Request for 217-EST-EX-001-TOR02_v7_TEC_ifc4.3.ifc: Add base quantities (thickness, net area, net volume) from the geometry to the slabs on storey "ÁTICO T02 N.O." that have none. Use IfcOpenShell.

First a look at what the model holds.

```python
import ifcopenshell
import ifcopenshell.util.element
import ifcopenshell.util.unit

model = ifcopenshell.open("217-EST-EX-001-TOR02_v7_TEC_ifc4.3.ifc")
print(model.schema)
for unit_type in ("LENGTHUNIT", "AREAUNIT", "VOLUMEUNIT"):
    print(unit_type, ifcopenshell.util.unit.calculate_unit_scale(model, unit_type))
storey = next(s for s in model.by_type("IfcBuildingStorey") if s.Name == "ÁTICO T02 N.O.")
slabs = [e for e in ifcopenshell.util.element.get_decomposition(storey) if e.is_a("IfcSlab")]
for e in sorted(slabs, key=lambda e: e.id()):
    print(e.id(), e.is_a(), e.Name, list(ifcopenshell.util.element.get_psets(e, qtos_only=True)), sep=" | ")
```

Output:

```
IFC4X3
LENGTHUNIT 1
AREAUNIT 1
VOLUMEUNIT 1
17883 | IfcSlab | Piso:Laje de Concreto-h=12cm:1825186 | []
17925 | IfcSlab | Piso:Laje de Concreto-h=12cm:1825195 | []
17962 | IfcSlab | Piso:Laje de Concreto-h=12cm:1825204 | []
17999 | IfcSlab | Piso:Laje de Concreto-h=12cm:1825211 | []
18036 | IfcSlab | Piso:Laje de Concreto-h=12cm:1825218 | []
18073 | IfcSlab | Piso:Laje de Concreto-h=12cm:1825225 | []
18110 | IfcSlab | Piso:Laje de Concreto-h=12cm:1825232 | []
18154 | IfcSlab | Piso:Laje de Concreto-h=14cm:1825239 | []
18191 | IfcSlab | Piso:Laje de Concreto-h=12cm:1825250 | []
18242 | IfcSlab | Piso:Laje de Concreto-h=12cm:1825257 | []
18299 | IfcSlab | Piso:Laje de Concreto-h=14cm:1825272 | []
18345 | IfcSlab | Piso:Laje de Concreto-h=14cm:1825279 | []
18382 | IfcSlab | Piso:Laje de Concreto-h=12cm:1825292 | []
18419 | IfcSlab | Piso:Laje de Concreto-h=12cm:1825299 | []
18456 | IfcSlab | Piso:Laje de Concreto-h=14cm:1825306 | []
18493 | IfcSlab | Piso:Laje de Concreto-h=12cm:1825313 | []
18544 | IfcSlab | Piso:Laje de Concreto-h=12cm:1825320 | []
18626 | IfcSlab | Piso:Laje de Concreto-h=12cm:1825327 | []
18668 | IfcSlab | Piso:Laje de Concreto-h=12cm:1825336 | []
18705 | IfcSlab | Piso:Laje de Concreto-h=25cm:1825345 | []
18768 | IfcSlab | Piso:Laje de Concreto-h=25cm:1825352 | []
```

```python
import ifcopenshell
import ifcopenshell.api.pset
import ifcopenshell.geom
import ifcopenshell.util.element
import ifcopenshell.util.shape
import ifcopenshell.util.unit

model = ifcopenshell.open("217-EST-EX-001-TOR02_v7_TEC_ifc4.3.ifc")
unit_scale = ifcopenshell.util.unit.calculate_unit_scale(model)
area_scale = ifcopenshell.util.unit.calculate_unit_scale(model, "AREAUNIT")
volume_scale = ifcopenshell.util.unit.calculate_unit_scale(model, "VOLUMEUNIT")
settings = ifcopenshell.geom.settings()

storey = next(s for s in model.by_type("IfcBuildingStorey") if s.Name == "ÁTICO T02 N.O.")
slabs = [e for e in ifcopenshell.util.element.get_decomposition(storey) if e.is_a("IfcSlab")]

for e in sorted(slabs, key=lambda e: e.id()):
    if ifcopenshell.util.element.get_psets(e, qtos_only=True, should_inherit=False):
        continue
    # Geometry comes back in metres, in the element's own axes.
    shape = ifcopenshell.geom.create_shape(settings, e)
    values = {
        "Width": ifcopenshell.util.shape.get_z(shape.geometry) / unit_scale,
        "NetArea": ifcopenshell.util.shape.get_footprint_area(shape.geometry) / area_scale,
        "NetVolume": ifcopenshell.util.shape.get_volume(shape.geometry) / volume_scale,
    }
    qto = ifcopenshell.api.pset.add_qto(model, product=e, name="Qto_SlabBaseQuantities")
    ifcopenshell.api.pset.edit_qto(model, qto=qto, properties=values)
    print(e.id(), {k: round(v, 3) for k, v in values.items()})

model.write("217-EST-EX-001-TOR02_v7_TEC_ifc4.3_updated.ifc")
```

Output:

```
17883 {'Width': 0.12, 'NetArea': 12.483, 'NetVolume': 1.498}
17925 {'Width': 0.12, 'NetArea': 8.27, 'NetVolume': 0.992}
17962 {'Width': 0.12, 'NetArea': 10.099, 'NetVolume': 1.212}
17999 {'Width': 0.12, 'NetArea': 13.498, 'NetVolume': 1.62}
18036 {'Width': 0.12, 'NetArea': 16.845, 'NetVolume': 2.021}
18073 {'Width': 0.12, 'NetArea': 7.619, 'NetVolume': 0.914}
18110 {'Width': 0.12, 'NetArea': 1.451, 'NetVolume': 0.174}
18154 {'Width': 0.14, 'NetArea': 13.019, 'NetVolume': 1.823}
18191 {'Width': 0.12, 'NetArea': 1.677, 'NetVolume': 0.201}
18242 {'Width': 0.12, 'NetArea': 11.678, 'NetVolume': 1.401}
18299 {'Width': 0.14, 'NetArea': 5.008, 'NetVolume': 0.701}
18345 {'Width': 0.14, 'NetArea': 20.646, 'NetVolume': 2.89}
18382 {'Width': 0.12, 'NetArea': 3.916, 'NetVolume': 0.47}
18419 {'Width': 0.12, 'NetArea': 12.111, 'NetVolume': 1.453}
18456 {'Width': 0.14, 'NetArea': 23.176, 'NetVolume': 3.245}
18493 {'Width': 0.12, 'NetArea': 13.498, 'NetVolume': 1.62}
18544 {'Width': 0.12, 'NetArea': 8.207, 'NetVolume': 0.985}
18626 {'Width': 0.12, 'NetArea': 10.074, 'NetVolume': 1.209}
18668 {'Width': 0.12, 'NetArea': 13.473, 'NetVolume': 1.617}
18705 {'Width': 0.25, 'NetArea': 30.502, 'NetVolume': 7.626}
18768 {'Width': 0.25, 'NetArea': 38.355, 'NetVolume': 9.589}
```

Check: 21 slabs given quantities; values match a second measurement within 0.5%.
